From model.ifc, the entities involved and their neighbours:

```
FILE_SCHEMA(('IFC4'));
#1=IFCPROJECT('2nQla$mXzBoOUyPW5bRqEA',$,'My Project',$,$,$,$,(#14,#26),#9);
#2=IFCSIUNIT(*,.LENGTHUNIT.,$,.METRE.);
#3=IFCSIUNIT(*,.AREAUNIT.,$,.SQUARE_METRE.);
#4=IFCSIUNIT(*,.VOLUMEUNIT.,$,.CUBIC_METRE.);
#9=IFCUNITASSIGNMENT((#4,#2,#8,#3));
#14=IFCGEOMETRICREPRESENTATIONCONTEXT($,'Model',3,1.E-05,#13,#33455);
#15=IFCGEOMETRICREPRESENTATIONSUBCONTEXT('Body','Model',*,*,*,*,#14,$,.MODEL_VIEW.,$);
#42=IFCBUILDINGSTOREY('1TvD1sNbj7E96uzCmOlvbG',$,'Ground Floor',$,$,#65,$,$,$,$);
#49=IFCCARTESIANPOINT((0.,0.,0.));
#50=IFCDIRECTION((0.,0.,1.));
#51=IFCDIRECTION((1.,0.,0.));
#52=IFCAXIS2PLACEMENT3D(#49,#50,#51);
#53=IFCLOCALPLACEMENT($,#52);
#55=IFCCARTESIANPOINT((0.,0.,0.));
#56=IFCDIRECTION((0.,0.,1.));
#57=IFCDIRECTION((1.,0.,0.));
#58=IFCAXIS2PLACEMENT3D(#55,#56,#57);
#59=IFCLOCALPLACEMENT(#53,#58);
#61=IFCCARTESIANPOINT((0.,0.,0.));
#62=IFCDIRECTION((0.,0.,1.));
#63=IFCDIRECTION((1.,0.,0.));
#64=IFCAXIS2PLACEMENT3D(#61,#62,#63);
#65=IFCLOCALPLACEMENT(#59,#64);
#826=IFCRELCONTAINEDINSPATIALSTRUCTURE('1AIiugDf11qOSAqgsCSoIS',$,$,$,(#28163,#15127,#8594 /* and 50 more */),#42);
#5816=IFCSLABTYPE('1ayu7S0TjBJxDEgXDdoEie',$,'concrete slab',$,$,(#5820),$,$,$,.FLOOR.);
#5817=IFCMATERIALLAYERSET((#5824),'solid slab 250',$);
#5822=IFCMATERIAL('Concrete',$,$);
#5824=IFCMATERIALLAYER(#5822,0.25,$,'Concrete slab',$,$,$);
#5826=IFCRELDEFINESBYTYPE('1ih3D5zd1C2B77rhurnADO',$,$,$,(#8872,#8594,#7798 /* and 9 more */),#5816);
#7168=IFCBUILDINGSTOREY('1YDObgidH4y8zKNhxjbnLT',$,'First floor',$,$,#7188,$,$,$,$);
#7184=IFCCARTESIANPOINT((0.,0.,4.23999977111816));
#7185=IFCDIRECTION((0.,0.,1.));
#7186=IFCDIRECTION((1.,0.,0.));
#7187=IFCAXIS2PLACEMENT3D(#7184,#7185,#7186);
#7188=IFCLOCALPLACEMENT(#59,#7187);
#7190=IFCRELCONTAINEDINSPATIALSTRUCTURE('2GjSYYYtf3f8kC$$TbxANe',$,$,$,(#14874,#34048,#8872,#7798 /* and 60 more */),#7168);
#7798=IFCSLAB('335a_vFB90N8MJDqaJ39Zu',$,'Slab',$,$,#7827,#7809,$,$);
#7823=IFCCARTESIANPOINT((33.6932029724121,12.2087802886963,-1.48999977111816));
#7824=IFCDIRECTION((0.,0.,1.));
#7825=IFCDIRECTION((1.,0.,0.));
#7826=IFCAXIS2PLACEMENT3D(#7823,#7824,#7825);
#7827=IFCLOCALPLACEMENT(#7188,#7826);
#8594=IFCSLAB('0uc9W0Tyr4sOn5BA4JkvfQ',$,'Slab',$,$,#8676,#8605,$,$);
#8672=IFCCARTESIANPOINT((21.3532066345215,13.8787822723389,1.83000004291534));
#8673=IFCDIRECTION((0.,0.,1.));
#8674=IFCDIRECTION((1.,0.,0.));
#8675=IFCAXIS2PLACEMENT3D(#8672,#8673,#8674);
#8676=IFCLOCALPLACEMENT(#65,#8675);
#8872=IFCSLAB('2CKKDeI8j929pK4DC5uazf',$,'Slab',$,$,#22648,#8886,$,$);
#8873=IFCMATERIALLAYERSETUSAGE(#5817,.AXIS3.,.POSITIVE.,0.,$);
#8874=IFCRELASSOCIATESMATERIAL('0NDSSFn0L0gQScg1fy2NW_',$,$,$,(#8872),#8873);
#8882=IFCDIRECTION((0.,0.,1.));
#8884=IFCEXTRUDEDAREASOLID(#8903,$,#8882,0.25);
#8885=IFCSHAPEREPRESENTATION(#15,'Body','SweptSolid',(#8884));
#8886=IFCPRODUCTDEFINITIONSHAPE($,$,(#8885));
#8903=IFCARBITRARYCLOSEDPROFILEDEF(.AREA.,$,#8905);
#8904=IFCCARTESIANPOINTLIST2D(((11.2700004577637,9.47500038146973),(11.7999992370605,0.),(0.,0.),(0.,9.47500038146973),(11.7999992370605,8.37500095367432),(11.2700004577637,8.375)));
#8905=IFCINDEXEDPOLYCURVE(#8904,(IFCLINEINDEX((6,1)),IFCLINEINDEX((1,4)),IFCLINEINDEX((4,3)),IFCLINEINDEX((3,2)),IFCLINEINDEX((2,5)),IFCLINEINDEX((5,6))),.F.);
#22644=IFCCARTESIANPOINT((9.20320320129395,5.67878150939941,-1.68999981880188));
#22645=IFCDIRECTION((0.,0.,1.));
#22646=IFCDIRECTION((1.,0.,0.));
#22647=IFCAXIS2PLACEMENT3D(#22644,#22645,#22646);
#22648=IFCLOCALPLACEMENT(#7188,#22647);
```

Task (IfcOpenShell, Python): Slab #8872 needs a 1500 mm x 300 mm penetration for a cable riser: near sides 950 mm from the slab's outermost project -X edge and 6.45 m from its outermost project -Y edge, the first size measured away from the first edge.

```python
import numpy as np
import ifcopenshell
import ifcopenshell.api.feature
import ifcopenshell.api.geometry
import ifcopenshell.api.root
import ifcopenshell.geom
import ifcopenshell.util.placement
import ifcopenshell.util.representation
import ifcopenshell.util.shape
import ifcopenshell.util.unit

model = ifcopenshell.open("model.ifc")
unit_scale = ifcopenshell.util.unit.calculate_unit_scale(model)
settings = ifcopenshell.geom.settings()


def volume(element):
    """Net volume in cubic metres, openings subtracted."""
    shape = ifcopenshell.geom.create_shape(settings, element)
    return ifcopenshell.util.shape.get_volume(shape.geometry)


slab = model.by_id(8872)
before = volume(slab)

# Extent in the slab's own axes, in metres. The edges named are its -X and -Y sides.
slab_shape = ifcopenshell.geom.create_shape(settings, slab)
vertices = ifcopenshell.util.shape.get_vertices(slab_shape.geometry)
x_min, y_min, bottom = vertices.min(axis=0)
top = vertices[:, 2].max()

opening = ifcopenshell.api.root.create_entity(model, ifc_class="IfcOpeningElement", name="Cable riser opening", predefined_type="OPENING")
context = ifcopenshell.util.representation.get_context(model, "Model", "Body", "MODEL_VIEW")
width, depth = 1.5, 0.3
outline = [(0.0, 0.0), (width, 0.0), (width, depth), (0.0, depth), (0.0, 0.0)]
# Overshoot both faces by 50 mm so the cut is clean.
shape = ifcopenshell.api.geometry.add_slab_representation(
    model, context=context, depth=top - bottom + 0.1, polyline=outline
)
ifcopenshell.api.geometry.assign_representation(model, product=opening, representation=shape)

matrix = ifcopenshell.util.placement.get_local_placement(slab.ObjectPlacement)
matrix[:, 3] = matrix @ np.append(np.array([x_min + 0.95, y_min + 6.45, bottom - 0.05]) / unit_scale, 1.0)
ifcopenshell.api.geometry.edit_object_placement(model, product=opening, matrix=matrix, is_si=False)
ifcopenshell.api.feature.add_feature(model, feature=opening, element=slab)

after = volume(slab)

print(f"slab volume {before:.3f} -> {after:.3f} m3")

model.write("model_v2.ifc")
```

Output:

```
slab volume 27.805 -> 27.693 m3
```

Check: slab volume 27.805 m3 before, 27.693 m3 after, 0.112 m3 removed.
